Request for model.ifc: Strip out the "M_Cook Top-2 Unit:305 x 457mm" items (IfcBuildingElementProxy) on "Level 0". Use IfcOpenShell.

First a look at what the model holds.

```python
import ifcopenshell
import ifcopenshell.util.element

model = ifcopenshell.open("model.ifc")
print(model.schema)
storey = next(s for s in model.by_type("IfcBuildingStorey") if s.Name == "Level 0")
proxies = [e for e in ifcopenshell.util.element.get_decomposition(storey) if e.is_a("IfcBuildingElementProxy")]
seen = {}
for e in proxies:
    element_type = ifcopenshell.util.element.get_type(e)
    name = element_type.Name if element_type not in (None, e) else None
    seen[name] = seen.get(name, 0) + 1
for name, count in sorted(seen.items(), key=str):
    print(count, "x", name)
```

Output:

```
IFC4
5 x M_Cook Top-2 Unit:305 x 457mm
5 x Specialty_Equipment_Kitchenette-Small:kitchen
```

```python
import ifcopenshell
import ifcopenshell.api.root
import ifcopenshell.util.element

model = ifcopenshell.open("model.ifc")

storey = next(s for s in model.by_type("IfcBuildingStorey") if s.Name == "Level 0")
proxies = [e for e in ifcopenshell.util.element.get_decomposition(storey) if e.is_a("IfcBuildingElementProxy")]
targets = [e for e in proxies if (t := ifcopenshell.util.element.get_type(e)) not in (None, e) and t.Name == "M_Cook Top-2 Unit:305 x 457mm"]

for e in targets:
    ifcopenshell.api.root.remove_product(model, product=e)
print(len(targets), "removed")

model.write("model-out.ifc")
```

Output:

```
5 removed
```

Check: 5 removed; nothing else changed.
